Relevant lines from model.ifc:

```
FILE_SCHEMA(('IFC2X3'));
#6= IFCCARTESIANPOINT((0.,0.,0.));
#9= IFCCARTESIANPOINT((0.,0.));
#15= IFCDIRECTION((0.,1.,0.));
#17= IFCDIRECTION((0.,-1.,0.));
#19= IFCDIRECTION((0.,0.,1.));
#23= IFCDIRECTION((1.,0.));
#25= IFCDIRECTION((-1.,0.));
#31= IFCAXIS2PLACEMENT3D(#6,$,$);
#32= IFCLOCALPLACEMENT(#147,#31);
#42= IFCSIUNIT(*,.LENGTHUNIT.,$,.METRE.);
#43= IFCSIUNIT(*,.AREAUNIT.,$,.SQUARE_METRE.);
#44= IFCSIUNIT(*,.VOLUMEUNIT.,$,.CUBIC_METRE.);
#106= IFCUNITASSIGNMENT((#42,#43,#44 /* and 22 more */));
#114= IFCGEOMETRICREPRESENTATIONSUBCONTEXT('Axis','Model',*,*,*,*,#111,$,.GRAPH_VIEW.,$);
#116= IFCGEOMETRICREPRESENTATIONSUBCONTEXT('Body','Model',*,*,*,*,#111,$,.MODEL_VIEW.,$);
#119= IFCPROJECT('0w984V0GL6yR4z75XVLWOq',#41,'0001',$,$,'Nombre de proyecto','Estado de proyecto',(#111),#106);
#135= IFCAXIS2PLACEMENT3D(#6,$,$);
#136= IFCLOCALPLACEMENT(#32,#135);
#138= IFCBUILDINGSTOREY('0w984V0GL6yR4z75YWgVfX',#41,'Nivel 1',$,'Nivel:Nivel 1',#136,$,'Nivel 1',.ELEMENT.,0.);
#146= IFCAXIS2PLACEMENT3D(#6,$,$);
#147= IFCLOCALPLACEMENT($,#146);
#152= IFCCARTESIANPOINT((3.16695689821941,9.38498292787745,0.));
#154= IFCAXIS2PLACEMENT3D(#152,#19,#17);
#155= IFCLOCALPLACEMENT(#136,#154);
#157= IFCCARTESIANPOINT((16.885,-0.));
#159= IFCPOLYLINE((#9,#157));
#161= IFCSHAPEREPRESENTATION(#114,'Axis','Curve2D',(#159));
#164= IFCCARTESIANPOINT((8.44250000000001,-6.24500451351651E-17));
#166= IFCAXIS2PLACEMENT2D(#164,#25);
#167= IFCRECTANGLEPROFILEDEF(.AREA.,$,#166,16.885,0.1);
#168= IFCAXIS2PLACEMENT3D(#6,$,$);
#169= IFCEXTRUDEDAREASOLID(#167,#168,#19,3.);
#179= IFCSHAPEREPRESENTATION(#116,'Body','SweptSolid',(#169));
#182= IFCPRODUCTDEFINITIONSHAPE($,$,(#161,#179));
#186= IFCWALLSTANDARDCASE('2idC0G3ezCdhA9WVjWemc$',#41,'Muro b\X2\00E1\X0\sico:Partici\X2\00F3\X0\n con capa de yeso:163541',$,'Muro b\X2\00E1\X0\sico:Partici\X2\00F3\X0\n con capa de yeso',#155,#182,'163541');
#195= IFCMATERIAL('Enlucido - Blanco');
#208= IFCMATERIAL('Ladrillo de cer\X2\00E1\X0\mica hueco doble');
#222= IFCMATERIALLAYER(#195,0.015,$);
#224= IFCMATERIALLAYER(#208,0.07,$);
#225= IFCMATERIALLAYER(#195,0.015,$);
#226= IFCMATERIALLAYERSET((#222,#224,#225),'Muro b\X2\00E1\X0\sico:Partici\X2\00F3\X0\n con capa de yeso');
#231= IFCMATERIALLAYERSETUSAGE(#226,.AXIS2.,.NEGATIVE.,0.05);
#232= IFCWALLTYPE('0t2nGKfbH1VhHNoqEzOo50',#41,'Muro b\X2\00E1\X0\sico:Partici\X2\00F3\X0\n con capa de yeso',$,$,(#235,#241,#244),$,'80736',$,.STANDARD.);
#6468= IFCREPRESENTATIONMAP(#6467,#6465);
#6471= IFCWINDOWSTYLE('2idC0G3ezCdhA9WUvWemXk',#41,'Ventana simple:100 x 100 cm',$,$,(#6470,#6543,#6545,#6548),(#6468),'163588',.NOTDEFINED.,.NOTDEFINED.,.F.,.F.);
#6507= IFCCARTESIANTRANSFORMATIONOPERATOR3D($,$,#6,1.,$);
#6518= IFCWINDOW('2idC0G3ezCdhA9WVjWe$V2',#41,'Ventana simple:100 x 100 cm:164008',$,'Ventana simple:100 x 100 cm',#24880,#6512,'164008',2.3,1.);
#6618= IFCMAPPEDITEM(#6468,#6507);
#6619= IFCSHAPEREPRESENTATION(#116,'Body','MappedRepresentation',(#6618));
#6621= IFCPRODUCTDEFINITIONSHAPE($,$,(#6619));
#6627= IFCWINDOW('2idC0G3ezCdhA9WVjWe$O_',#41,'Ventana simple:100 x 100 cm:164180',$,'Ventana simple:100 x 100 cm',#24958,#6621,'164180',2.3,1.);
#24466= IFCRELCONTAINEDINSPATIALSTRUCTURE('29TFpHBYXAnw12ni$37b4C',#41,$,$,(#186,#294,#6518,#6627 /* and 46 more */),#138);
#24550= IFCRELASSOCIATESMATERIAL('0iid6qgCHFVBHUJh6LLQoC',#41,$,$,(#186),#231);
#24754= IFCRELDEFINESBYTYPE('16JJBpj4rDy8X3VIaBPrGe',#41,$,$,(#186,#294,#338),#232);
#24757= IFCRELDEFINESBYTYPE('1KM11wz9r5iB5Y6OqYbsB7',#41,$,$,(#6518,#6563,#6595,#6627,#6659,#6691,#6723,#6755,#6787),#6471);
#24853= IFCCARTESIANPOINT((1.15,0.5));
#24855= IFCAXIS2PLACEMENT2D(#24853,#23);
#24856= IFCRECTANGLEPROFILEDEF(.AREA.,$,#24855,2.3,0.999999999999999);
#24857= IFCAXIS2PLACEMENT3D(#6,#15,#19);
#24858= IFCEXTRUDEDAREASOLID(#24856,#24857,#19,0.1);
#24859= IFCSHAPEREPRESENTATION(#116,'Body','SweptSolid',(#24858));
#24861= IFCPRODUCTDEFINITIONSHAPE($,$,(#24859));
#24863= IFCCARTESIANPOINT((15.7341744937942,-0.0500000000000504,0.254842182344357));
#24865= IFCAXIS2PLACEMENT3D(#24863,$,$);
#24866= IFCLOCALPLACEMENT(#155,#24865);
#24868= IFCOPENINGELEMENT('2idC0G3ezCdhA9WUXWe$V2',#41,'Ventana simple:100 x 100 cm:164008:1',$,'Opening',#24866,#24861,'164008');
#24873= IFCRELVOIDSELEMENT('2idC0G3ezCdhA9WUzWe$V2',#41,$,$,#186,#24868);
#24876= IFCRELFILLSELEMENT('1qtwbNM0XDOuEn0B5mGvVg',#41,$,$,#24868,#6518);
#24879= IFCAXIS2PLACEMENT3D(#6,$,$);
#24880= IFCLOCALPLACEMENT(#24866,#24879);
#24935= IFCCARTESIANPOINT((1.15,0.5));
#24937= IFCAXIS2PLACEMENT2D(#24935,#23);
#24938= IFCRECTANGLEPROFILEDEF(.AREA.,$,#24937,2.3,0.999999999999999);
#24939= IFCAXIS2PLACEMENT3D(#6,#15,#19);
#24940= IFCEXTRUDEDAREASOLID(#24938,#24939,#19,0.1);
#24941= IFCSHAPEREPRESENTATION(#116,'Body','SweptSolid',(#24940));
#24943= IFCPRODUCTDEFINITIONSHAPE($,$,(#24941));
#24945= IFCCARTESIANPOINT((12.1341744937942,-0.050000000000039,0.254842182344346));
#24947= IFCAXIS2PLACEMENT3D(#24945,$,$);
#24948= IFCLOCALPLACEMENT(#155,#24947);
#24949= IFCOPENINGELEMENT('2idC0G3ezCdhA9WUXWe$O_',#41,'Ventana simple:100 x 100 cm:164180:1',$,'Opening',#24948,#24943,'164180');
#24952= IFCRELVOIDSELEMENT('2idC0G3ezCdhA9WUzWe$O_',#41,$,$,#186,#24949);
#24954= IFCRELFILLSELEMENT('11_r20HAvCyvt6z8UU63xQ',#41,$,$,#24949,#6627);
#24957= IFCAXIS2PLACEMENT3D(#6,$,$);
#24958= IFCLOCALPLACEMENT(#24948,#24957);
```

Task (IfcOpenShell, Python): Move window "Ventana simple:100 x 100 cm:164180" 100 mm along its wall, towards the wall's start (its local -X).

```python
import ifcopenshell
import ifcopenshell.api.geometry
import ifcopenshell.util.placement
import ifcopenshell.util.unit

model = ifcopenshell.open("model.ifc")
unit_scale = ifcopenshell.util.unit.calculate_unit_scale(model)

window = model.by_guid("2idC0G3ezCdhA9WVjWe$O_")
opening = window.FillsVoids[0].RelatingOpeningElement
wall = opening.VoidsElements[0].RelatingBuildingElement

wall_matrix = ifcopenshell.util.placement.get_local_placement(wall.ObjectPlacement)
shift = wall_matrix[:3, 0] * -0.1 / unit_scale
before = ifcopenshell.util.placement.get_local_placement(window.ObjectPlacement)[:3, 3].copy()

# The window is placed relative to its opening, so it follows when the opening moves.
matrix = ifcopenshell.util.placement.get_local_placement(opening.ObjectPlacement)
matrix[:3, 3] += shift
ifcopenshell.api.geometry.edit_object_placement(
    model, product=opening, matrix=matrix, is_si=False, should_transform_children=True
)

after = ifcopenshell.util.placement.get_local_placement(window.ObjectPlacement)[:3, 3]
print("window moved by", (after - before).round(3) + 0.0)

model.write("model_edited.ifc")
```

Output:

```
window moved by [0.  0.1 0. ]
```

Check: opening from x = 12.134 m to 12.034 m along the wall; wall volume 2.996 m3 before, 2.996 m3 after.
